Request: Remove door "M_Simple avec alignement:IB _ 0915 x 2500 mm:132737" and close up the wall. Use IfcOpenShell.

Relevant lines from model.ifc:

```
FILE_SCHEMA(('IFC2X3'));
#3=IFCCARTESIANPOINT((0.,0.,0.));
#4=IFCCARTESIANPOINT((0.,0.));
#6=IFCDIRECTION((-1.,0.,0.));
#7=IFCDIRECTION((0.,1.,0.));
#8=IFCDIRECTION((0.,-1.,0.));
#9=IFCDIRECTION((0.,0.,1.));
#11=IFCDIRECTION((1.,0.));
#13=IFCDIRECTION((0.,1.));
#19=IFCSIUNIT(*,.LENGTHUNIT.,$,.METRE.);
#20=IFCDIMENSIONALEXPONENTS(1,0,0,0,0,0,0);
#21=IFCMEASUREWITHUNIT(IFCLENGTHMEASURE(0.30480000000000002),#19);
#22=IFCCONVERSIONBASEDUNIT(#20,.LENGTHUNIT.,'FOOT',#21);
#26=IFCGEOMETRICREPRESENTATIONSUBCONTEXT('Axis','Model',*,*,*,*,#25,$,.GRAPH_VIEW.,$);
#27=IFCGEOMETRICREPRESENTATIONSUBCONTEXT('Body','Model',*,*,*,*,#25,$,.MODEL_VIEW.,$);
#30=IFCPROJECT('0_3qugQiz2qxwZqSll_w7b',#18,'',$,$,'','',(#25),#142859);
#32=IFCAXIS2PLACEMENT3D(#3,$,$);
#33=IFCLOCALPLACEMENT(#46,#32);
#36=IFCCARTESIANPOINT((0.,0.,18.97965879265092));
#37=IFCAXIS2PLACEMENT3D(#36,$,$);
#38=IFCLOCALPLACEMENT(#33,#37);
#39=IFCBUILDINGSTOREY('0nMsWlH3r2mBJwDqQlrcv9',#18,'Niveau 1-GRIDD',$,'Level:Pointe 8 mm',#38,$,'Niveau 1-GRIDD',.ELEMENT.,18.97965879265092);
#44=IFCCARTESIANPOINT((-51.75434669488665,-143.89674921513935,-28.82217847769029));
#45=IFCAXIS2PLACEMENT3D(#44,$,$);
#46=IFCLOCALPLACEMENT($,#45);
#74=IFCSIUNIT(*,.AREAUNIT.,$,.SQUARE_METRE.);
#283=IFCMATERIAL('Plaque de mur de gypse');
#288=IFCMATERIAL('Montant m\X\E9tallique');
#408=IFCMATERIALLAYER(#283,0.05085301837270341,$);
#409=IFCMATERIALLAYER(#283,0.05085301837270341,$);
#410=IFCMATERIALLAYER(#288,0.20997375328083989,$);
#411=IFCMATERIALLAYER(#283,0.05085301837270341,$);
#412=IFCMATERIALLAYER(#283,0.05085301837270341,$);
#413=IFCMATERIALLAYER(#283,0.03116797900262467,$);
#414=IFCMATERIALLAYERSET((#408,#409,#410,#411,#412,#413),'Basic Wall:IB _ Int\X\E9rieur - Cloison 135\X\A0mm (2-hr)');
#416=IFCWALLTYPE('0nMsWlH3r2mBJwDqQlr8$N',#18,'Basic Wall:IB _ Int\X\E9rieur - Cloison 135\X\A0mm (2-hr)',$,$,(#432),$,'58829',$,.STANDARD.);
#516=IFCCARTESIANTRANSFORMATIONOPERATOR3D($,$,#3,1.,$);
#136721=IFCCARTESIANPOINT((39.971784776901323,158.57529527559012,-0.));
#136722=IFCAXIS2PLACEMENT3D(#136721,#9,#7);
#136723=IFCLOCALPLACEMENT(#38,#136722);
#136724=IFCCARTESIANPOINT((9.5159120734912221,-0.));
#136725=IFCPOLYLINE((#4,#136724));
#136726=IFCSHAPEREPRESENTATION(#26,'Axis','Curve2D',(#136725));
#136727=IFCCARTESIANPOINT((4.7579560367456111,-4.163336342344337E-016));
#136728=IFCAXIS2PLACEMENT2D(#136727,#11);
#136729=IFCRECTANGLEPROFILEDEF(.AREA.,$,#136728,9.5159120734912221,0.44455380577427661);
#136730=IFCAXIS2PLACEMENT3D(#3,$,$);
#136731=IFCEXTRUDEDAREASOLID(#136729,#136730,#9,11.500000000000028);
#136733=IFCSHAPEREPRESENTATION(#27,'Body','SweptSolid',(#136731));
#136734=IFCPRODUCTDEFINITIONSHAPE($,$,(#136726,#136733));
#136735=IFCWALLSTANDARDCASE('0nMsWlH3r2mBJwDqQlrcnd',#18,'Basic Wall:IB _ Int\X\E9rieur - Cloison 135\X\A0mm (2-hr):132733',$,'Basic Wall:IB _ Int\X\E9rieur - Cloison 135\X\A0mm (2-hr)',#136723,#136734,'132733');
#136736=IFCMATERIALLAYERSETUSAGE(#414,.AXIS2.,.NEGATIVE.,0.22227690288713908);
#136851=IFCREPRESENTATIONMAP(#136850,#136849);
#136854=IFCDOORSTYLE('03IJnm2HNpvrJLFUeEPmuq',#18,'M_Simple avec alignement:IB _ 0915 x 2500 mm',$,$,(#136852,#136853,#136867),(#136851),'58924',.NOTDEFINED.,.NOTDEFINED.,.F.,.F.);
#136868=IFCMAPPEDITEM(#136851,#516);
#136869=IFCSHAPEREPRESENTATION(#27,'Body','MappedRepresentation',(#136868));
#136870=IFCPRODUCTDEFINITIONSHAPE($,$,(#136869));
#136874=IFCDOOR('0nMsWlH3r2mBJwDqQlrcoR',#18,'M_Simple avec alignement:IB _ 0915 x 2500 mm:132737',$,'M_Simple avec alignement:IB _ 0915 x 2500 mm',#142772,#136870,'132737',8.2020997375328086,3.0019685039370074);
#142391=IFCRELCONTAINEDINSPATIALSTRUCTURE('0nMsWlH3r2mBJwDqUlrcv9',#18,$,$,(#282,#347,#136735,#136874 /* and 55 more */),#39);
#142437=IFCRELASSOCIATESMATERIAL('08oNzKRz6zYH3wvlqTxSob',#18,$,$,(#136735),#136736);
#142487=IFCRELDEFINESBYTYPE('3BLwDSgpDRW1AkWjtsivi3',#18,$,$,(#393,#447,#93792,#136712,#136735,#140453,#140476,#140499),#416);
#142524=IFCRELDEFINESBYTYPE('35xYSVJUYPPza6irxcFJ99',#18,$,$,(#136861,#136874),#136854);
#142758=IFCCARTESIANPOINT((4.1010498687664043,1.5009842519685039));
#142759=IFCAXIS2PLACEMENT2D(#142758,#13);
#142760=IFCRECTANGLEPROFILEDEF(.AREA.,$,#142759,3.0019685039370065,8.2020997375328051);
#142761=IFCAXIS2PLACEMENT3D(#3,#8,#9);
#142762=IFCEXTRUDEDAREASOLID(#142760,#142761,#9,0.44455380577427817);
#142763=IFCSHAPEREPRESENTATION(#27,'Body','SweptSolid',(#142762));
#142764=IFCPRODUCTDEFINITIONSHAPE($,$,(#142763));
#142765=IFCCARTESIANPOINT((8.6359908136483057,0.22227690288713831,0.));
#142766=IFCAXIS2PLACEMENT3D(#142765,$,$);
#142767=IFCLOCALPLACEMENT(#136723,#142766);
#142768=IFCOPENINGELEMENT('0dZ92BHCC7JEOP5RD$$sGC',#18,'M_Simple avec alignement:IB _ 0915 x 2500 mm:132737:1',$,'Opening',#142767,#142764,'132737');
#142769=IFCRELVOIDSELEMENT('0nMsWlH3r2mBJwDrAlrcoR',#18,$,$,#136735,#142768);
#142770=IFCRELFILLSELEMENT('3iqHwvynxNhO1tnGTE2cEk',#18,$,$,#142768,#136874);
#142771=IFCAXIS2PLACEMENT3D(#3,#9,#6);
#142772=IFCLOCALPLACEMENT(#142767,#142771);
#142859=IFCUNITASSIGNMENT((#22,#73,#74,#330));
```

```python
import ifcopenshell
import ifcopenshell.api.feature
import ifcopenshell.api.root
import ifcopenshell.geom
import ifcopenshell.util.shape

model = ifcopenshell.open("model.ifc")
settings = ifcopenshell.geom.settings()


def volume(element):
    """Net volume in cubic metres, openings subtracted."""
    shape = ifcopenshell.geom.create_shape(settings, element)
    return ifcopenshell.util.shape.get_volume(shape.geometry)


door = model.by_guid("0nMsWlH3r2mBJwDqQlrcoR")
opening = door.FillsVoids[0].RelatingOpeningElement
wall = opening.VoidsElements[0].RelatingBuildingElement
before = volume(wall)

ifcopenshell.api.root.remove_product(model, product=door)
ifcopenshell.api.feature.remove_feature(model, feature=opening)

after = volume(wall)

print(f"wall volume {before:.3f} -> {after:.3f} m3")

model.write("model_updated.ifc")
```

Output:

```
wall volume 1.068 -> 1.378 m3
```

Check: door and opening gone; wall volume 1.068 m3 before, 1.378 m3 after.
